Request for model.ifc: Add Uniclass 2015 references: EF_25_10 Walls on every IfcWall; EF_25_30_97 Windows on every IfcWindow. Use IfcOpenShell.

First a look at what the model holds.

```python
import ifcopenshell

model = ifcopenshell.open("model.ifc")
print(model.schema)
print("classifications:", [c.Name for c in model.by_type("IfcClassification")])
for ifc_class in ("IfcDoor", "IfcRoof", "IfcStair", "IfcWall", "IfcWindow"):
    print(ifc_class, len(model.by_type(ifc_class)))
```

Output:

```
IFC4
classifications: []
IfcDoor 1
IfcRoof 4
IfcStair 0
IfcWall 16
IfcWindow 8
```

```python
import ifcopenshell
import ifcopenshell.api.classification

model = ifcopenshell.open("model.ifc")

system = ifcopenshell.api.classification.add_classification(model, classification="Uniclass 2015")

codes = {
    "IfcWall": ("EF_25_10", "Walls"),
    "IfcWindow": ("EF_25_30_97", "Windows"),
}
for ifc_class, (code, name) in codes.items():
    products = model.by_type(ifc_class)
    ifcopenshell.api.classification.add_reference(
        model, products=products, classification=system, identification=code, name=name
    )
    print(code, len(products))

model.write("model_rev.ifc")
```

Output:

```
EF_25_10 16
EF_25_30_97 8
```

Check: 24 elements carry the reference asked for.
